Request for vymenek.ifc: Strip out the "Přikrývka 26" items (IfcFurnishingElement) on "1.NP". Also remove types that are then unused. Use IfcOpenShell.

First a look at what the model holds.

```python
import ifcopenshell
import ifcopenshell.util.element

model = ifcopenshell.open("vymenek.ifc")
print(model.schema)
storey = next(s for s in model.by_type("IfcBuildingStorey") if s.Name == "1.NP")
furniture = [e for e in ifcopenshell.util.element.get_decomposition(storey) if e.is_a("IfcFurnishingElement")]
seen = {}
for e in furniture:
    element_type = ifcopenshell.util.element.get_type(e)
    name = element_type.Name if element_type not in (None, e) else None
    seen[name] = seen.get(name, 0) + 1
for name, count in sorted(seen.items(), key=str):
    print(count, "x", name)
```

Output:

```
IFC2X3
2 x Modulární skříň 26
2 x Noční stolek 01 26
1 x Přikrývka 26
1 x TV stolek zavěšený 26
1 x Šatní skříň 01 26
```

```python
import ifcopenshell
import ifcopenshell.api.root
import ifcopenshell.util.element

model = ifcopenshell.open("vymenek.ifc")

storey = next(s for s in model.by_type("IfcBuildingStorey") if s.Name == "1.NP")
furniture = [e for e in ifcopenshell.util.element.get_decomposition(storey) if e.is_a("IfcFurnishingElement")]
targets = [e for e in furniture if (t := ifcopenshell.util.element.get_type(e)) not in (None, e) and t.Name == "Přikrývka 26"]
types = {ifcopenshell.util.element.get_type(e) for e in targets} - {None, *targets}

for e in targets:
    ifcopenshell.api.root.remove_product(model, product=e)
print(len(targets), "removed")

unused = [t for t in types if not ifcopenshell.util.element.get_types(t)]
for t in unused:
    ifcopenshell.api.root.remove_product(model, product=t)
print(len(unused), "unused types removed")

model.write("vymenek-out.ifc")
```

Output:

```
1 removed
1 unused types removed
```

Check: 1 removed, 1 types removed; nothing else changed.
